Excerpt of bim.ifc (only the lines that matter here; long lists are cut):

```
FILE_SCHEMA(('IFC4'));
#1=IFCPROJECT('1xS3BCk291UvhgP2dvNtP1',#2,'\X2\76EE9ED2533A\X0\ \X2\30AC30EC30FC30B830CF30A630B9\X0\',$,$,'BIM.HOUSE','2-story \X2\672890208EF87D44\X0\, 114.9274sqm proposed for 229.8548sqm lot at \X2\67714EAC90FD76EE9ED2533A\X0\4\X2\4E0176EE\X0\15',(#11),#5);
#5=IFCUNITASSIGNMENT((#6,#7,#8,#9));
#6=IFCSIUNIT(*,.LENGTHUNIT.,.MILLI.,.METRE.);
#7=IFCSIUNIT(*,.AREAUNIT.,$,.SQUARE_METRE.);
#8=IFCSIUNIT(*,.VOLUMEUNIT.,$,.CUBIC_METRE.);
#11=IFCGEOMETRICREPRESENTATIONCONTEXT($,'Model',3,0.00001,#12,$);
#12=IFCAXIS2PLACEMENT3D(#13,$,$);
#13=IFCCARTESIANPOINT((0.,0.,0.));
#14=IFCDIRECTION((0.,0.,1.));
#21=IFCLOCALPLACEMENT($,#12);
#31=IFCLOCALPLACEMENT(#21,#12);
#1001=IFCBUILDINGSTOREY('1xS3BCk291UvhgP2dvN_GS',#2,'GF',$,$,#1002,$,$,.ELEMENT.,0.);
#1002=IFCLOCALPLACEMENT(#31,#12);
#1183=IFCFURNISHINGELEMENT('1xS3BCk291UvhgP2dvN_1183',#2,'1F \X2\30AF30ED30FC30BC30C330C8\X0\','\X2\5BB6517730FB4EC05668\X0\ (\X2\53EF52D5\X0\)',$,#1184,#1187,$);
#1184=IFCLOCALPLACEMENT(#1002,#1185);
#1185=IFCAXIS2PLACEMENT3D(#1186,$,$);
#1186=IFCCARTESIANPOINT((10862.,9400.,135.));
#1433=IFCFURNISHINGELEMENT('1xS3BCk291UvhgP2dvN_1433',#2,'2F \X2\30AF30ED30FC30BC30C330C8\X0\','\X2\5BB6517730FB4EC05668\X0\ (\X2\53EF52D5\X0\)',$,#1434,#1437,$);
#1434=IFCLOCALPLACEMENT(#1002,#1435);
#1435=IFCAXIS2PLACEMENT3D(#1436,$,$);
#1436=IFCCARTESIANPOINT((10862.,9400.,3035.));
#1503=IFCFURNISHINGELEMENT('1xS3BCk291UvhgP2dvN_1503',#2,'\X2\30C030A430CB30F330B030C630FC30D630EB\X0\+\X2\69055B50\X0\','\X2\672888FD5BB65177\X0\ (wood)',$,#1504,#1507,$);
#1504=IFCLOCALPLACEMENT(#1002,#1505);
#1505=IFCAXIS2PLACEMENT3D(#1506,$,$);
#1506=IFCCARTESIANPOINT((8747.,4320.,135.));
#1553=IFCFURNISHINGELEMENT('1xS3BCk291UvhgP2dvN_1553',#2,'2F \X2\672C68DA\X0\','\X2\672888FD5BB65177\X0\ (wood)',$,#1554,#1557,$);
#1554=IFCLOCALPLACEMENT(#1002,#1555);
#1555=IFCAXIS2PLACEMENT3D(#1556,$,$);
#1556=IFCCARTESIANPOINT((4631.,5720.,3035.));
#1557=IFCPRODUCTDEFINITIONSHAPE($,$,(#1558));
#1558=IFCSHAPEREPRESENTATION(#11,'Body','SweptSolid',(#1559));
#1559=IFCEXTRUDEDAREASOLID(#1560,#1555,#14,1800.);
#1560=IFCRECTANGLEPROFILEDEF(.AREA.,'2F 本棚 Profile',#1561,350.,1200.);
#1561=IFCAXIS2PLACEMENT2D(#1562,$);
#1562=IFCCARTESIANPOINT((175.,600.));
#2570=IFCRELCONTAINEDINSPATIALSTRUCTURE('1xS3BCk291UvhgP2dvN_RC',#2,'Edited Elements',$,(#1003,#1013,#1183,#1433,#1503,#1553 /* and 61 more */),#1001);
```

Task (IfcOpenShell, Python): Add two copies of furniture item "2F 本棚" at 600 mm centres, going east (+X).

```python
import numpy as np
import ifcopenshell
import ifcopenshell.api.geometry
import ifcopenshell.api.root
import ifcopenshell.util.element
import ifcopenshell.util.placement

model = ifcopenshell.open("bim.ifc")


def reuse_history(source, copy):
    """copy_class also copies each property set's owner history, people and application; keep the originals."""
    for rel in copy.IsDefinedBy:
        if rel.is_a("IfcRelDefinesByProperties") and (history := rel.RelatingPropertyDefinition.OwnerHistory):
            rel.RelatingPropertyDefinition.OwnerHistory = source.OwnerHistory
            ifcopenshell.util.element.remove_deep2(model, history)


source = model.by_guid("1xS3BCk291UvhgP2dvN_1553")
base = ifcopenshell.util.placement.get_local_placement(source.ObjectPlacement)
step = np.array([1.0, 0.0, 0.0]) * 600.0

for i in range(1, 3):
    copy = ifcopenshell.api.root.copy_class(model, product=source)
    copy.Representation = ifcopenshell.util.element.copy_deep(
        model, source.Representation, exclude=["IfcGeometricRepresentationContext", "IfcRepresentationMap"]
    )
    reuse_history(source, copy)
    matrix = base.copy()
    matrix[:3, 3] += i * step
    print("added at", matrix[:3, 3].round(3) + 0.0)
    ifcopenshell.api.geometry.edit_object_placement(model, product=copy, matrix=matrix, is_si=False)

model.write("bim_edited.ifc")
```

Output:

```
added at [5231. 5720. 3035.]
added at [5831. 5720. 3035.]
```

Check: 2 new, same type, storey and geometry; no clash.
